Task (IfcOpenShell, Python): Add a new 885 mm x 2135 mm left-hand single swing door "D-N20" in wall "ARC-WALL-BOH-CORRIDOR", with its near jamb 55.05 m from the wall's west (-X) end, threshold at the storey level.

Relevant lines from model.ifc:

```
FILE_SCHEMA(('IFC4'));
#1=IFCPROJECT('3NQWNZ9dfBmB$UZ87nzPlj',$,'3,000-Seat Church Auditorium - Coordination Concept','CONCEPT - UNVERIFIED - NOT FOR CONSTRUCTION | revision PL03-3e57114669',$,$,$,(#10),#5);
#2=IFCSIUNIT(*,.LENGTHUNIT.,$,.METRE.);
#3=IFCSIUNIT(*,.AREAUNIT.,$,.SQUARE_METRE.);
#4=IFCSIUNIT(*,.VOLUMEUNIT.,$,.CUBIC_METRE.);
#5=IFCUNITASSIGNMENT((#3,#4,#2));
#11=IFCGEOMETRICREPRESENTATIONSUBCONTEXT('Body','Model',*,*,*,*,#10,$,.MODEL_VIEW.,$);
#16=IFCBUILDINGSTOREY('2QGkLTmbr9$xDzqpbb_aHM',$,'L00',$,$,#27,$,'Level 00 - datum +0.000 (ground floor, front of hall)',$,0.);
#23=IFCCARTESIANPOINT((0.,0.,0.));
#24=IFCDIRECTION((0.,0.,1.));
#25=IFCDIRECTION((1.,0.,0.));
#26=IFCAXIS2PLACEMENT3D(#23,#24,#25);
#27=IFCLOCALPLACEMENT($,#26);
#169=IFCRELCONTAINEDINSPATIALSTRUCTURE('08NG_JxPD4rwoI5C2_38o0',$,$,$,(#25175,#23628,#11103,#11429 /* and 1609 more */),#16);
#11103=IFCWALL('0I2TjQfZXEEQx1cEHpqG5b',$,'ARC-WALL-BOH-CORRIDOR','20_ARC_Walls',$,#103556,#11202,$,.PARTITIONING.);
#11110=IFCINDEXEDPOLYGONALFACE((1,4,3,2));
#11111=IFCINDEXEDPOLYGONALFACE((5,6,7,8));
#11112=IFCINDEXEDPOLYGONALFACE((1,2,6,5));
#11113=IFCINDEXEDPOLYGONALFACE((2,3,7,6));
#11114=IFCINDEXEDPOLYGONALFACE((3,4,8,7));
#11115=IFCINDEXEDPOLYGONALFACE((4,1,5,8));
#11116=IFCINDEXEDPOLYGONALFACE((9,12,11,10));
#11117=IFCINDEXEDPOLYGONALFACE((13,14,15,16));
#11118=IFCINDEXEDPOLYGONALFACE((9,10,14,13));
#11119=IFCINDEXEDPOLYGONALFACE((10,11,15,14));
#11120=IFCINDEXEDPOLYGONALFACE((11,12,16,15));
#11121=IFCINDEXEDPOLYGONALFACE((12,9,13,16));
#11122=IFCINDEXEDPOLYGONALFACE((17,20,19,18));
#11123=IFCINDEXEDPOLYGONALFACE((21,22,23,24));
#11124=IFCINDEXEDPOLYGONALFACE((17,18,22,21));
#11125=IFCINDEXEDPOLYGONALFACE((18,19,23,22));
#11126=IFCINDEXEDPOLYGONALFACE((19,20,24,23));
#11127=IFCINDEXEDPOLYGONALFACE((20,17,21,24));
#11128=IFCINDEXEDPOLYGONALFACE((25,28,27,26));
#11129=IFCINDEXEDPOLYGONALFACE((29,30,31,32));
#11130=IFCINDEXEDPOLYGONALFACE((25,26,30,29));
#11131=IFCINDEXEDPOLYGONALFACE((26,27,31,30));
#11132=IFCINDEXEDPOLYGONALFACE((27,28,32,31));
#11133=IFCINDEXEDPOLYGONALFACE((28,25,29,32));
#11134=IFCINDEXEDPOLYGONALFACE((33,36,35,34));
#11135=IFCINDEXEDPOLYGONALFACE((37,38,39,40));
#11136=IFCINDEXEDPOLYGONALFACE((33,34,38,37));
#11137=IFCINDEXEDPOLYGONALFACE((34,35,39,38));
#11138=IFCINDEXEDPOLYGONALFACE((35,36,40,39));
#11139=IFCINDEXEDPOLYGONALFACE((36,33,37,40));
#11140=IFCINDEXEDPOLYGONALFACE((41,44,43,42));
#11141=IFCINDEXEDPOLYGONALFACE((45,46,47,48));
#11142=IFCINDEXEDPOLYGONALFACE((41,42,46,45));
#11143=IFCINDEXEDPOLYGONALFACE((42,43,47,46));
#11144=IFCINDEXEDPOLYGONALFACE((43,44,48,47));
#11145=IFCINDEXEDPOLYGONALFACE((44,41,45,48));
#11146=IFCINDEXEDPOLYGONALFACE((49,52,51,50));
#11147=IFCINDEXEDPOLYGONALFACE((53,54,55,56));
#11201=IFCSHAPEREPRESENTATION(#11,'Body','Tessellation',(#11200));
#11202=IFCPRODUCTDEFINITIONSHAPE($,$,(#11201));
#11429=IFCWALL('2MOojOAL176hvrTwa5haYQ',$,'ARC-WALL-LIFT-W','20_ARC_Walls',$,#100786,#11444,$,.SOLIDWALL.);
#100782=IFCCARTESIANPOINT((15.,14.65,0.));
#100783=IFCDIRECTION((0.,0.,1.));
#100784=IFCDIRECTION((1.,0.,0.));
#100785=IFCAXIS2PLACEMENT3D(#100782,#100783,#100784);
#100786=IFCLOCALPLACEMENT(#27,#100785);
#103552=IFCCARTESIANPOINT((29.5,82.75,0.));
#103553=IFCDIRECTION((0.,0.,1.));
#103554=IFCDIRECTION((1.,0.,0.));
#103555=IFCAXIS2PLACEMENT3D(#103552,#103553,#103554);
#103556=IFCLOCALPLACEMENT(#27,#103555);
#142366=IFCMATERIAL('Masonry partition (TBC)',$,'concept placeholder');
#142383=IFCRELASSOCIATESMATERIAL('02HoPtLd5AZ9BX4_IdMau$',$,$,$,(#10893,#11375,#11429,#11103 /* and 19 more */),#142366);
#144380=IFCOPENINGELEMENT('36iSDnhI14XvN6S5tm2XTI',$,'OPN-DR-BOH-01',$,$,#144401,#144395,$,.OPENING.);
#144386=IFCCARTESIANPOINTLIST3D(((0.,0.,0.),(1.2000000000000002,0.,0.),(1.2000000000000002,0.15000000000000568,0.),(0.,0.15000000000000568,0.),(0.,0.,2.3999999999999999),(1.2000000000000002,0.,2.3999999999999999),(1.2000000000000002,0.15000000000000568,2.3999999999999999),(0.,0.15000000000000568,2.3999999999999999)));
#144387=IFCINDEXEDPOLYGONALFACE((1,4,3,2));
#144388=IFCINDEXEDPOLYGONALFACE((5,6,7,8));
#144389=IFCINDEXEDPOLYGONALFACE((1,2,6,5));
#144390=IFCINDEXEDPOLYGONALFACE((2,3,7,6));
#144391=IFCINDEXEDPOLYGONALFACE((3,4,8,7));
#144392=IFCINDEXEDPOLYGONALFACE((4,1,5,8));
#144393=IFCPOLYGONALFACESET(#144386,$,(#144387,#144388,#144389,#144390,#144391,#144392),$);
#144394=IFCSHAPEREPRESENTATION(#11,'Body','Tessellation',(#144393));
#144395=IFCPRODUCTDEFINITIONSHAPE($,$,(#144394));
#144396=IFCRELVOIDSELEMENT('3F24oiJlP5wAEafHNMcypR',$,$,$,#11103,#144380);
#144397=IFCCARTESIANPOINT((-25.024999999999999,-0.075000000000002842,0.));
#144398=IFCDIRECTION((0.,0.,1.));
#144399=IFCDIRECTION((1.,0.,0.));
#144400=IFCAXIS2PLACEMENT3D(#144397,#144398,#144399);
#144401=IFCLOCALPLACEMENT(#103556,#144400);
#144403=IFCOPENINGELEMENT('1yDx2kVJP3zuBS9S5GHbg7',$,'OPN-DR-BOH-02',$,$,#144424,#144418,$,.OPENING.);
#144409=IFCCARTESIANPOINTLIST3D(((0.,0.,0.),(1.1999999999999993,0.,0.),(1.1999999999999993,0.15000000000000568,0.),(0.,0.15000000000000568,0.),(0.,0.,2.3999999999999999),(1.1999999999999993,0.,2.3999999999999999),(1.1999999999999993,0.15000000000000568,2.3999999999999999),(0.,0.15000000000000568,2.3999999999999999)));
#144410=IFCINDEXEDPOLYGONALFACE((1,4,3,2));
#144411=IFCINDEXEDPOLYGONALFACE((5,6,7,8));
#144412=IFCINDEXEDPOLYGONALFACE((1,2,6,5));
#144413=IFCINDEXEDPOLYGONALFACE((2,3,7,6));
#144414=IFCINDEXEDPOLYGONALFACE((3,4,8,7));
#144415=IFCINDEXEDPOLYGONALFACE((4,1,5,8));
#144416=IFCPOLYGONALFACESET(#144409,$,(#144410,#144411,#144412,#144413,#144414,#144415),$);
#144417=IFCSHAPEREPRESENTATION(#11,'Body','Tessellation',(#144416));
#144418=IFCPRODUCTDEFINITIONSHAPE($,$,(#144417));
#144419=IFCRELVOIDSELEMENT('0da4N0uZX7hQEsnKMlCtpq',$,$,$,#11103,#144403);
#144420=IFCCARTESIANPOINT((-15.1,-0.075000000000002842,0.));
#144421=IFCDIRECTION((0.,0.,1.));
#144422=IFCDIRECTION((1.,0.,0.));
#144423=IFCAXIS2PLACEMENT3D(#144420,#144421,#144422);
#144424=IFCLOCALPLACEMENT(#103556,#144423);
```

```python
import numpy as np
import ifcopenshell
import ifcopenshell.api.feature
import ifcopenshell.api.geometry
import ifcopenshell.api.root
import ifcopenshell.api.spatial
import ifcopenshell.geom
import ifcopenshell.util.element
import ifcopenshell.util.placement
import ifcopenshell.util.representation
import ifcopenshell.util.shape
import ifcopenshell.util.unit

model = ifcopenshell.open("model.ifc")
unit_scale = ifcopenshell.util.unit.calculate_unit_scale(model)
settings = ifcopenshell.geom.settings()


def volume(element):
    """Net volume in cubic metres, openings subtracted."""
    shape = ifcopenshell.geom.create_shape(settings, element)
    return ifcopenshell.util.shape.get_volume(shape.geometry)


wall = model.by_guid("0I2TjQfZXEEQx1cEHpqG5b")
storey = ifcopenshell.util.element.get_container(wall, ifc_class="IfcBuildingStorey")
context = ifcopenshell.util.representation.get_context(model, "Model", "Body", "MODEL_VIEW")
before = volume(wall)

width, height, from_end, sill = 0.885, 2.135, 55.05, 0.0  # metres

# The wall runs along its own X axis, and the end named is its -X end.
wall_shape = ifcopenshell.geom.create_shape(settings, wall)
x, y, z = ifcopenshell.util.shape.get_vertices(wall_shape.geometry).T
start = x.min() + from_end
face, thickness = float(y.min()), float(y.max() - y.min())
wall_matrix = ifcopenshell.util.placement.get_local_placement(wall.ObjectPlacement)
level = ifcopenshell.util.placement.get_local_placement(storey.ObjectPlacement)[2, 3]


def in_wall(x, y):
    """Placement at x, y metres in the wall's axes, at sill height."""
    matrix = wall_matrix.copy()
    matrix[:, 3] = wall_matrix @ np.array([x / unit_scale, y / unit_scale, 0.0, 1.0])
    matrix[2, 3] = level + sill / unit_scale
    return matrix


# Opening: a box that overshoots both wall faces by 50 mm.
opening = ifcopenshell.api.root.create_entity(model, ifc_class="IfcOpeningElement", predefined_type="OPENING")
box = ifcopenshell.api.geometry.add_wall_representation(
    model, context=context, length=width, height=height, thickness=thickness + 0.1
)
ifcopenshell.api.geometry.assign_representation(model, product=opening, representation=box)
ifcopenshell.api.geometry.edit_object_placement(model, product=opening, matrix=in_wall(start, face - 0.05), is_si=False)
ifcopenshell.api.feature.add_feature(model, feature=opening, element=wall)

door = ifcopenshell.api.root.create_entity(model, ifc_class="IfcDoor", name="D-N20", predefined_type="DOOR")
door.OverallWidth, door.OverallHeight = width / unit_scale, height / unit_scale
door.OperationType = "SINGLE_SWING_LEFT"
body = ifcopenshell.api.geometry.add_door_representation(
    model,
    context=context,
    overall_width=door.OverallWidth,
    overall_height=door.OverallHeight,
    operation_type="SINGLE_SWING_LEFT",
    lining_properties={"LiningDepth": thickness / unit_scale, "ThresholdDepth": thickness / unit_scale},
)
ifcopenshell.api.geometry.assign_representation(model, product=door, representation=body)
ifcopenshell.api.spatial.assign_container(model, products=[door], relating_structure=storey)
ifcopenshell.api.feature.add_filling(model, opening=opening, element=door)

# The lining spans the wall, so the door starts at the wall face.
ifcopenshell.api.geometry.edit_object_placement(model, product=door, matrix=in_wall(start, face), is_si=False)

after = volume(wall)

print(f"wall volume {before:.3f} -> {after:.3f} m3")

model.write("model_rev.ifc")
```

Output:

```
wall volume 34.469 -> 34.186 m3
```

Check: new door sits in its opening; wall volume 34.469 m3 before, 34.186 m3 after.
